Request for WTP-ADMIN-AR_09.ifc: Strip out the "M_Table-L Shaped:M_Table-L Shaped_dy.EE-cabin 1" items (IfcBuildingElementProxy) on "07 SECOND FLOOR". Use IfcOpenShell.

First a look at what the model holds.

```python
import ifcopenshell
import ifcopenshell.util.element

model = ifcopenshell.open("WTP-ADMIN-AR_09.ifc")
print(model.schema)
storey = next(s for s in model.by_type("IfcBuildingStorey") if s.Name == "07 SECOND FLOOR")
proxies = [e for e in ifcopenshell.util.element.get_decomposition(storey) if e.is_a("IfcBuildingElementProxy")]
seen = {}
for e in proxies:
    element_type = ifcopenshell.util.element.get_type(e)
    name = element_type.Name if element_type not in (None, e) else None
    seen[name] = seen.get(name, 0) + 1
for name, count in sorted(seen.items(), key=str):
    print(count, "x", name)
```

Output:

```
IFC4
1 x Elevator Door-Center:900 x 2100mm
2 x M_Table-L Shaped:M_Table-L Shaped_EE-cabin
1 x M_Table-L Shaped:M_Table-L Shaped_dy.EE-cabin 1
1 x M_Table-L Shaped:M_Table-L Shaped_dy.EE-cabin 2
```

```python
import ifcopenshell
import ifcopenshell.api.root
import ifcopenshell.util.element

model = ifcopenshell.open("WTP-ADMIN-AR_09.ifc")

storey = next(s for s in model.by_type("IfcBuildingStorey") if s.Name == "07 SECOND FLOOR")
proxies = [e for e in ifcopenshell.util.element.get_decomposition(storey) if e.is_a("IfcBuildingElementProxy")]
targets = [e for e in proxies if (t := ifcopenshell.util.element.get_type(e)) not in (None, e) and t.Name == "M_Table-L Shaped:M_Table-L Shaped_dy.EE-cabin 1"]

for e in targets:
    ifcopenshell.api.root.remove_product(model, product=e)
print(len(targets), "removed")

model.write("WTP-ADMIN-AR_09_edited.ifc")
```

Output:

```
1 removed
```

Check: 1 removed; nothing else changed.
